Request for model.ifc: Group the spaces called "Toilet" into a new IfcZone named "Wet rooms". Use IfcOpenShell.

First a look at what the model holds.

```python
import ifcopenshell

model = ifcopenshell.open("model.ifc")
print(model.schema)
seen = {}
for space in model.by_type("IfcSpace"):
    seen[space.LongName] = seen.get(space.LongName, 0) + 1
for name, count in sorted(seen.items(), key=str):
    print(count, "x", name)
print("zones:", [z.Name for z in model.by_type("IfcZone")][:20])
```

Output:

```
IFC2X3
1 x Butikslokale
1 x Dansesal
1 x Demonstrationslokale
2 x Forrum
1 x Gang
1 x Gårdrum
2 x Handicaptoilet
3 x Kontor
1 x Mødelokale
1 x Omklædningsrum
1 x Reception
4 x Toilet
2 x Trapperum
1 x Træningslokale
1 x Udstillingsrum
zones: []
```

```python
import ifcopenshell
import ifcopenshell.api.group
import ifcopenshell.api.root

model = ifcopenshell.open("model.ifc")

names = {"Toilet"}
spaces = [s for s in model.by_type("IfcSpace") if s.LongName in names]

zone = ifcopenshell.api.root.create_entity(model, ifc_class="IfcZone", name="Wet rooms")
ifcopenshell.api.group.assign_group(model, products=spaces, group=zone)
print(len(spaces), "spaces in", zone.Name)

model.write("model_rev.ifc")
```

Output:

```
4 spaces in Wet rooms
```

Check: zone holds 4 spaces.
